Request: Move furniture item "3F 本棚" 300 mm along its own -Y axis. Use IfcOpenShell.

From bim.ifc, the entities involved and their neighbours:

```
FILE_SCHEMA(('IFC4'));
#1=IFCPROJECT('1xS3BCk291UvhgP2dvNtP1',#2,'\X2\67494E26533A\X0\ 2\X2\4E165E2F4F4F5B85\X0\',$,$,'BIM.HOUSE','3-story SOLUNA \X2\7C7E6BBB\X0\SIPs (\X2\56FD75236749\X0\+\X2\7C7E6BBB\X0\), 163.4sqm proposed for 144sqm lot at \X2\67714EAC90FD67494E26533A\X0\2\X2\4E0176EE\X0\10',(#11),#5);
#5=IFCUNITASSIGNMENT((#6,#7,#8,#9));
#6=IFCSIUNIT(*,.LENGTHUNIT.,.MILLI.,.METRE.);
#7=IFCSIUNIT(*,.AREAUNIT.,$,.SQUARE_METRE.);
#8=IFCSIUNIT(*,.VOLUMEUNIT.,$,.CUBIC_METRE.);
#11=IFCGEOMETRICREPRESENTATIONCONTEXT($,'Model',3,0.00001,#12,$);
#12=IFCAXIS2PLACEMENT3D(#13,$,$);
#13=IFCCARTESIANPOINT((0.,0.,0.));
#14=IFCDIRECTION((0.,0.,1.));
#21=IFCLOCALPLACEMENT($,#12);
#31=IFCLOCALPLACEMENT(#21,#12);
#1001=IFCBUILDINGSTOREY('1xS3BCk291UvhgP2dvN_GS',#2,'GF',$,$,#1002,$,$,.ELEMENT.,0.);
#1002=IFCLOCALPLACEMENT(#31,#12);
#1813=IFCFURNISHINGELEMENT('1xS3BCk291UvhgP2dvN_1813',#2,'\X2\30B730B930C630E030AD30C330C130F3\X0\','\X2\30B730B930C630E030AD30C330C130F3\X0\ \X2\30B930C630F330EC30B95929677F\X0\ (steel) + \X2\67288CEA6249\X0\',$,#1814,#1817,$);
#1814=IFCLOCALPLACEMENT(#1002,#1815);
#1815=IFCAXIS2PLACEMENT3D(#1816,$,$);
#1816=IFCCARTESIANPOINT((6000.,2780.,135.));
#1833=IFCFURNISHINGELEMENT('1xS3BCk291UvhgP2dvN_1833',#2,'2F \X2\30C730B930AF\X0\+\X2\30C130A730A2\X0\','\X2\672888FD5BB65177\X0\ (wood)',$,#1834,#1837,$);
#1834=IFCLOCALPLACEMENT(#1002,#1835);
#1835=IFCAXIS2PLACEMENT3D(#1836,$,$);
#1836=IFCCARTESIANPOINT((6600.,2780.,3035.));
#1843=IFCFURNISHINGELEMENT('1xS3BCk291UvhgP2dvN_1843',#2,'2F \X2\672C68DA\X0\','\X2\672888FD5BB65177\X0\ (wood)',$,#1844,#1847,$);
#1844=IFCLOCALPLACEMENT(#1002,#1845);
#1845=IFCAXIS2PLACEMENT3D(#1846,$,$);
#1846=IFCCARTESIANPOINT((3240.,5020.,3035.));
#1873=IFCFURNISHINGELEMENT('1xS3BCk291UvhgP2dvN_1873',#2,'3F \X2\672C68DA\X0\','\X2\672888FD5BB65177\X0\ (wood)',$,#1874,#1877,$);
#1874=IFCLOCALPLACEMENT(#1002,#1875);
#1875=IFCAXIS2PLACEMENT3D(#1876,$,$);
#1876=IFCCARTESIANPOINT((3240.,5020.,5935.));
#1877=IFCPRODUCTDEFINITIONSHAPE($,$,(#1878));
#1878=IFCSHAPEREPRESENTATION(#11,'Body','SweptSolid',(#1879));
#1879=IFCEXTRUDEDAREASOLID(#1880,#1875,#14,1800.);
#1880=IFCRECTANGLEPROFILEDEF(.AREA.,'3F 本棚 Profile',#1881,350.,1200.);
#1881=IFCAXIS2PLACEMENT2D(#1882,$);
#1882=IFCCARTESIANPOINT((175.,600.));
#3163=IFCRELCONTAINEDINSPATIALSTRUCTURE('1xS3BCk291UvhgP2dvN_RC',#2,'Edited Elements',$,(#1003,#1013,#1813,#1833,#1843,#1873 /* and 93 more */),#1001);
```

```python
import ifcopenshell
import ifcopenshell.api.geometry
import ifcopenshell.util.placement

model = ifcopenshell.open("bim.ifc")

item = model.by_id(1873)
matrix = ifcopenshell.util.placement.get_local_placement(item.ObjectPlacement)
matrix[:3, 3] -= matrix[:3, 1] * 300.0
ifcopenshell.api.geometry.edit_object_placement(model, product=item, matrix=matrix, is_si=False)

print(ifcopenshell.util.placement.get_local_placement(item.ObjectPlacement).round(3) + 0.0)

model.write("bim_updated.ifc")
```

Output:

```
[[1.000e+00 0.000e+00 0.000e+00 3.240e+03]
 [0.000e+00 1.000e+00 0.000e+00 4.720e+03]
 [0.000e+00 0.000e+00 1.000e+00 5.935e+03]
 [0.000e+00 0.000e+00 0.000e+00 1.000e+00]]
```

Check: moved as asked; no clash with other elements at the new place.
